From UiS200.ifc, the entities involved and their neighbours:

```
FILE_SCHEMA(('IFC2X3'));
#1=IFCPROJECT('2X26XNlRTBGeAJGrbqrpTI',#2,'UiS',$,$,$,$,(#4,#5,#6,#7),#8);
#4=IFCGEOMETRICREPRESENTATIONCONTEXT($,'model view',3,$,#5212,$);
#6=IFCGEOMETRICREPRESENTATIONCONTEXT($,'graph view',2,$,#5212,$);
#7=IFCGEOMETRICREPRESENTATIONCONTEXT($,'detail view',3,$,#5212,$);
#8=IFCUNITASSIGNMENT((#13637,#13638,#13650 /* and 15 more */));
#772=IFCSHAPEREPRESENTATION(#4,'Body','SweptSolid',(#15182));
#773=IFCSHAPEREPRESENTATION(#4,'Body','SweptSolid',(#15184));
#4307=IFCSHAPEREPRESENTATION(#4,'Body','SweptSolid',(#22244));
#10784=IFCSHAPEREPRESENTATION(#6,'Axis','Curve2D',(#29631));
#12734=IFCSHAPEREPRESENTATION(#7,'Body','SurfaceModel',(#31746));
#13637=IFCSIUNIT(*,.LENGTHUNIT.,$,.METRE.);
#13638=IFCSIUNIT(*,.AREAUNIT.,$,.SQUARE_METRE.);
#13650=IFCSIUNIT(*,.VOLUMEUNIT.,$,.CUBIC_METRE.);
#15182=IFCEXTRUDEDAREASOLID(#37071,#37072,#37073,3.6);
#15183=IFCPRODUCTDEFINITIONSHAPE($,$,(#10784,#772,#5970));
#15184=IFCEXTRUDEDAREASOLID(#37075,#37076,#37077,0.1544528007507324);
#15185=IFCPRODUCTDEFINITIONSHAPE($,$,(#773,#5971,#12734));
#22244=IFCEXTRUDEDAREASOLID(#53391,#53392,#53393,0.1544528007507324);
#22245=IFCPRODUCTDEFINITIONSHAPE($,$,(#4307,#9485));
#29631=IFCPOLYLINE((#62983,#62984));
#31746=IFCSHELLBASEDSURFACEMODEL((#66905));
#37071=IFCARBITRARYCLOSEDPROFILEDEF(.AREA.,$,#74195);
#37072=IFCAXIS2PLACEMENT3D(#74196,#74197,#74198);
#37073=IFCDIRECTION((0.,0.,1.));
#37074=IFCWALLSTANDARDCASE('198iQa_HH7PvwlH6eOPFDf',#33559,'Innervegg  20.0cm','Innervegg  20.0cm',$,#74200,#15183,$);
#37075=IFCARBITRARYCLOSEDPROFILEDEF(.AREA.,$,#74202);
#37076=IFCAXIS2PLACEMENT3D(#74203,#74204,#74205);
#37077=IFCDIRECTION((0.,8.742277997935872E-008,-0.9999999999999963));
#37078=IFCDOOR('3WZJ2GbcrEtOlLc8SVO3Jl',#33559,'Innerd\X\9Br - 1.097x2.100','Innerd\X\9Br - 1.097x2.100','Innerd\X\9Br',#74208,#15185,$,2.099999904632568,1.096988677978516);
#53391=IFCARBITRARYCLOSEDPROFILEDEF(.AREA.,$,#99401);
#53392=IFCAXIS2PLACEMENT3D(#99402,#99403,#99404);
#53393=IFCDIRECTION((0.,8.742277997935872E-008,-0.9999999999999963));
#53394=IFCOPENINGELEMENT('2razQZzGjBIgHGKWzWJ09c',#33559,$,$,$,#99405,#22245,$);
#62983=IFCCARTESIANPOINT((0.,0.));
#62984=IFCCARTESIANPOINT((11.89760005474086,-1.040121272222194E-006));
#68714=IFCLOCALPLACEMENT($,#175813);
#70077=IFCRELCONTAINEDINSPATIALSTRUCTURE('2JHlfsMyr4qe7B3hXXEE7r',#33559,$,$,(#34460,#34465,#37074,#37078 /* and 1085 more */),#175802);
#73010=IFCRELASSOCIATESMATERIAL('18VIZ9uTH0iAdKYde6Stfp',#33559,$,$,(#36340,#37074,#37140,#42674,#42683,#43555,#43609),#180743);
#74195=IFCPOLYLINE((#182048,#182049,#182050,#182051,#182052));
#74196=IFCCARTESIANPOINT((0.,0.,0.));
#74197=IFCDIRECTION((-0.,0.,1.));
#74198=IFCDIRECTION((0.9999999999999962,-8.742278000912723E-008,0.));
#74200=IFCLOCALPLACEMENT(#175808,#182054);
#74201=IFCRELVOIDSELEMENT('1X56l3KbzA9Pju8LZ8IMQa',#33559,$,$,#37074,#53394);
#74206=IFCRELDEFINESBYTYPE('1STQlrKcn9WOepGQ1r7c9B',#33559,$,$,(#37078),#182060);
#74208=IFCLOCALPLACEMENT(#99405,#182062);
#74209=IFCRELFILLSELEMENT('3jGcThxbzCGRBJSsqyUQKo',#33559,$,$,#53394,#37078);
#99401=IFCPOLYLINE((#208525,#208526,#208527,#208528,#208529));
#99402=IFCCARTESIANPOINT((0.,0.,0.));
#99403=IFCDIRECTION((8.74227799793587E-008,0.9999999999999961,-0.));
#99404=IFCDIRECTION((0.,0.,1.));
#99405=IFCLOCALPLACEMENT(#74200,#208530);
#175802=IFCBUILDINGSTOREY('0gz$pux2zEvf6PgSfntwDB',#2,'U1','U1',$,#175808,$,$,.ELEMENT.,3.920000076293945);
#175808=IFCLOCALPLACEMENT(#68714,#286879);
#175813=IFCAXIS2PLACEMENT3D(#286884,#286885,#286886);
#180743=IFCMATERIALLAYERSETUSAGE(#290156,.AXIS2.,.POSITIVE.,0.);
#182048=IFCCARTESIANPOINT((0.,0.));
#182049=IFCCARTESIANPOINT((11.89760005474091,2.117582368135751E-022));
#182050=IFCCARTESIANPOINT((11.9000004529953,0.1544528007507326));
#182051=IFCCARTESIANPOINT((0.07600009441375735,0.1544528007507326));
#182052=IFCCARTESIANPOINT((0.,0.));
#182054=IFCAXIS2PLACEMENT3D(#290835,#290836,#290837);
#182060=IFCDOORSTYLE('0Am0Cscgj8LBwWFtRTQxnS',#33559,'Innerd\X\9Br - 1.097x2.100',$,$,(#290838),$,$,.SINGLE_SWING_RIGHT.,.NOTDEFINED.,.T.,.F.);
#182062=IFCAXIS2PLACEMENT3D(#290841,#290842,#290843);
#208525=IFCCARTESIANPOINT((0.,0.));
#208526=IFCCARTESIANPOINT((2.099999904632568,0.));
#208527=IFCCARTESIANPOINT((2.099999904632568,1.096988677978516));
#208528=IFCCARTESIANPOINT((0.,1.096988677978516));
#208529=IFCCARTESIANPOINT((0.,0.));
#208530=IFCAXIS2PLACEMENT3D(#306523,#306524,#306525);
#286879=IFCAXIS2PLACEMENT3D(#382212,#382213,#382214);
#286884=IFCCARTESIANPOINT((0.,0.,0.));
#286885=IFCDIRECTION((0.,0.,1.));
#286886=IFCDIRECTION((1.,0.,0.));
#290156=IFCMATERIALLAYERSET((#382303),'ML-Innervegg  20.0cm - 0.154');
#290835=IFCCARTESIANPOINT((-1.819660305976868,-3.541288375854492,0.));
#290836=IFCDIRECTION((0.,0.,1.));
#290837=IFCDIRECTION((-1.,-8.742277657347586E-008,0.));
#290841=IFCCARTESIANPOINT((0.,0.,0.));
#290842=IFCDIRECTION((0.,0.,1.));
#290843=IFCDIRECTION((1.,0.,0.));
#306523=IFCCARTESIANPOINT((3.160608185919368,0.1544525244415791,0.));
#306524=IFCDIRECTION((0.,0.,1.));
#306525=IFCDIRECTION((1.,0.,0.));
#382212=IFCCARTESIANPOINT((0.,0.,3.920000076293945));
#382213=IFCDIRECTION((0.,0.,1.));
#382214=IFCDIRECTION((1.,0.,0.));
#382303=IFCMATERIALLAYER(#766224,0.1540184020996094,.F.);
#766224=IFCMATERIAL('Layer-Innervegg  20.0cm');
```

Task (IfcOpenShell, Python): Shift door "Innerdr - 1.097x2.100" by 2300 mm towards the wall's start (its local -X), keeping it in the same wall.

```python
import ifcopenshell
import ifcopenshell.api.geometry
import ifcopenshell.util.placement
import ifcopenshell.util.unit

model = ifcopenshell.open("UiS200.ifc")
unit_scale = ifcopenshell.util.unit.calculate_unit_scale(model)

door = model.by_guid("3WZJ2GbcrEtOlLc8SVO3Jl")
opening = door.FillsVoids[0].RelatingOpeningElement
wall = opening.VoidsElements[0].RelatingBuildingElement

wall_matrix = ifcopenshell.util.placement.get_local_placement(wall.ObjectPlacement)
shift = wall_matrix[:3, 0] * -2.3 / unit_scale
before = ifcopenshell.util.placement.get_local_placement(door.ObjectPlacement)[:3, 3].copy()

# The door is placed relative to its opening, so it follows when the opening moves.
matrix = ifcopenshell.util.placement.get_local_placement(opening.ObjectPlacement)
matrix[:3, 3] += shift
ifcopenshell.api.geometry.edit_object_placement(
    model, product=opening, matrix=matrix, is_si=False, should_transform_children=True
)

after = ifcopenshell.util.placement.get_local_placement(door.ObjectPlacement)[:3, 3]
print("door moved by", (after - before).round(3) + 0.0)

model.write("UiS200_rev.ifc")
```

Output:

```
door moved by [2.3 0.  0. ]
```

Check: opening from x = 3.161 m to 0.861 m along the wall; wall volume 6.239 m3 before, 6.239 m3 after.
